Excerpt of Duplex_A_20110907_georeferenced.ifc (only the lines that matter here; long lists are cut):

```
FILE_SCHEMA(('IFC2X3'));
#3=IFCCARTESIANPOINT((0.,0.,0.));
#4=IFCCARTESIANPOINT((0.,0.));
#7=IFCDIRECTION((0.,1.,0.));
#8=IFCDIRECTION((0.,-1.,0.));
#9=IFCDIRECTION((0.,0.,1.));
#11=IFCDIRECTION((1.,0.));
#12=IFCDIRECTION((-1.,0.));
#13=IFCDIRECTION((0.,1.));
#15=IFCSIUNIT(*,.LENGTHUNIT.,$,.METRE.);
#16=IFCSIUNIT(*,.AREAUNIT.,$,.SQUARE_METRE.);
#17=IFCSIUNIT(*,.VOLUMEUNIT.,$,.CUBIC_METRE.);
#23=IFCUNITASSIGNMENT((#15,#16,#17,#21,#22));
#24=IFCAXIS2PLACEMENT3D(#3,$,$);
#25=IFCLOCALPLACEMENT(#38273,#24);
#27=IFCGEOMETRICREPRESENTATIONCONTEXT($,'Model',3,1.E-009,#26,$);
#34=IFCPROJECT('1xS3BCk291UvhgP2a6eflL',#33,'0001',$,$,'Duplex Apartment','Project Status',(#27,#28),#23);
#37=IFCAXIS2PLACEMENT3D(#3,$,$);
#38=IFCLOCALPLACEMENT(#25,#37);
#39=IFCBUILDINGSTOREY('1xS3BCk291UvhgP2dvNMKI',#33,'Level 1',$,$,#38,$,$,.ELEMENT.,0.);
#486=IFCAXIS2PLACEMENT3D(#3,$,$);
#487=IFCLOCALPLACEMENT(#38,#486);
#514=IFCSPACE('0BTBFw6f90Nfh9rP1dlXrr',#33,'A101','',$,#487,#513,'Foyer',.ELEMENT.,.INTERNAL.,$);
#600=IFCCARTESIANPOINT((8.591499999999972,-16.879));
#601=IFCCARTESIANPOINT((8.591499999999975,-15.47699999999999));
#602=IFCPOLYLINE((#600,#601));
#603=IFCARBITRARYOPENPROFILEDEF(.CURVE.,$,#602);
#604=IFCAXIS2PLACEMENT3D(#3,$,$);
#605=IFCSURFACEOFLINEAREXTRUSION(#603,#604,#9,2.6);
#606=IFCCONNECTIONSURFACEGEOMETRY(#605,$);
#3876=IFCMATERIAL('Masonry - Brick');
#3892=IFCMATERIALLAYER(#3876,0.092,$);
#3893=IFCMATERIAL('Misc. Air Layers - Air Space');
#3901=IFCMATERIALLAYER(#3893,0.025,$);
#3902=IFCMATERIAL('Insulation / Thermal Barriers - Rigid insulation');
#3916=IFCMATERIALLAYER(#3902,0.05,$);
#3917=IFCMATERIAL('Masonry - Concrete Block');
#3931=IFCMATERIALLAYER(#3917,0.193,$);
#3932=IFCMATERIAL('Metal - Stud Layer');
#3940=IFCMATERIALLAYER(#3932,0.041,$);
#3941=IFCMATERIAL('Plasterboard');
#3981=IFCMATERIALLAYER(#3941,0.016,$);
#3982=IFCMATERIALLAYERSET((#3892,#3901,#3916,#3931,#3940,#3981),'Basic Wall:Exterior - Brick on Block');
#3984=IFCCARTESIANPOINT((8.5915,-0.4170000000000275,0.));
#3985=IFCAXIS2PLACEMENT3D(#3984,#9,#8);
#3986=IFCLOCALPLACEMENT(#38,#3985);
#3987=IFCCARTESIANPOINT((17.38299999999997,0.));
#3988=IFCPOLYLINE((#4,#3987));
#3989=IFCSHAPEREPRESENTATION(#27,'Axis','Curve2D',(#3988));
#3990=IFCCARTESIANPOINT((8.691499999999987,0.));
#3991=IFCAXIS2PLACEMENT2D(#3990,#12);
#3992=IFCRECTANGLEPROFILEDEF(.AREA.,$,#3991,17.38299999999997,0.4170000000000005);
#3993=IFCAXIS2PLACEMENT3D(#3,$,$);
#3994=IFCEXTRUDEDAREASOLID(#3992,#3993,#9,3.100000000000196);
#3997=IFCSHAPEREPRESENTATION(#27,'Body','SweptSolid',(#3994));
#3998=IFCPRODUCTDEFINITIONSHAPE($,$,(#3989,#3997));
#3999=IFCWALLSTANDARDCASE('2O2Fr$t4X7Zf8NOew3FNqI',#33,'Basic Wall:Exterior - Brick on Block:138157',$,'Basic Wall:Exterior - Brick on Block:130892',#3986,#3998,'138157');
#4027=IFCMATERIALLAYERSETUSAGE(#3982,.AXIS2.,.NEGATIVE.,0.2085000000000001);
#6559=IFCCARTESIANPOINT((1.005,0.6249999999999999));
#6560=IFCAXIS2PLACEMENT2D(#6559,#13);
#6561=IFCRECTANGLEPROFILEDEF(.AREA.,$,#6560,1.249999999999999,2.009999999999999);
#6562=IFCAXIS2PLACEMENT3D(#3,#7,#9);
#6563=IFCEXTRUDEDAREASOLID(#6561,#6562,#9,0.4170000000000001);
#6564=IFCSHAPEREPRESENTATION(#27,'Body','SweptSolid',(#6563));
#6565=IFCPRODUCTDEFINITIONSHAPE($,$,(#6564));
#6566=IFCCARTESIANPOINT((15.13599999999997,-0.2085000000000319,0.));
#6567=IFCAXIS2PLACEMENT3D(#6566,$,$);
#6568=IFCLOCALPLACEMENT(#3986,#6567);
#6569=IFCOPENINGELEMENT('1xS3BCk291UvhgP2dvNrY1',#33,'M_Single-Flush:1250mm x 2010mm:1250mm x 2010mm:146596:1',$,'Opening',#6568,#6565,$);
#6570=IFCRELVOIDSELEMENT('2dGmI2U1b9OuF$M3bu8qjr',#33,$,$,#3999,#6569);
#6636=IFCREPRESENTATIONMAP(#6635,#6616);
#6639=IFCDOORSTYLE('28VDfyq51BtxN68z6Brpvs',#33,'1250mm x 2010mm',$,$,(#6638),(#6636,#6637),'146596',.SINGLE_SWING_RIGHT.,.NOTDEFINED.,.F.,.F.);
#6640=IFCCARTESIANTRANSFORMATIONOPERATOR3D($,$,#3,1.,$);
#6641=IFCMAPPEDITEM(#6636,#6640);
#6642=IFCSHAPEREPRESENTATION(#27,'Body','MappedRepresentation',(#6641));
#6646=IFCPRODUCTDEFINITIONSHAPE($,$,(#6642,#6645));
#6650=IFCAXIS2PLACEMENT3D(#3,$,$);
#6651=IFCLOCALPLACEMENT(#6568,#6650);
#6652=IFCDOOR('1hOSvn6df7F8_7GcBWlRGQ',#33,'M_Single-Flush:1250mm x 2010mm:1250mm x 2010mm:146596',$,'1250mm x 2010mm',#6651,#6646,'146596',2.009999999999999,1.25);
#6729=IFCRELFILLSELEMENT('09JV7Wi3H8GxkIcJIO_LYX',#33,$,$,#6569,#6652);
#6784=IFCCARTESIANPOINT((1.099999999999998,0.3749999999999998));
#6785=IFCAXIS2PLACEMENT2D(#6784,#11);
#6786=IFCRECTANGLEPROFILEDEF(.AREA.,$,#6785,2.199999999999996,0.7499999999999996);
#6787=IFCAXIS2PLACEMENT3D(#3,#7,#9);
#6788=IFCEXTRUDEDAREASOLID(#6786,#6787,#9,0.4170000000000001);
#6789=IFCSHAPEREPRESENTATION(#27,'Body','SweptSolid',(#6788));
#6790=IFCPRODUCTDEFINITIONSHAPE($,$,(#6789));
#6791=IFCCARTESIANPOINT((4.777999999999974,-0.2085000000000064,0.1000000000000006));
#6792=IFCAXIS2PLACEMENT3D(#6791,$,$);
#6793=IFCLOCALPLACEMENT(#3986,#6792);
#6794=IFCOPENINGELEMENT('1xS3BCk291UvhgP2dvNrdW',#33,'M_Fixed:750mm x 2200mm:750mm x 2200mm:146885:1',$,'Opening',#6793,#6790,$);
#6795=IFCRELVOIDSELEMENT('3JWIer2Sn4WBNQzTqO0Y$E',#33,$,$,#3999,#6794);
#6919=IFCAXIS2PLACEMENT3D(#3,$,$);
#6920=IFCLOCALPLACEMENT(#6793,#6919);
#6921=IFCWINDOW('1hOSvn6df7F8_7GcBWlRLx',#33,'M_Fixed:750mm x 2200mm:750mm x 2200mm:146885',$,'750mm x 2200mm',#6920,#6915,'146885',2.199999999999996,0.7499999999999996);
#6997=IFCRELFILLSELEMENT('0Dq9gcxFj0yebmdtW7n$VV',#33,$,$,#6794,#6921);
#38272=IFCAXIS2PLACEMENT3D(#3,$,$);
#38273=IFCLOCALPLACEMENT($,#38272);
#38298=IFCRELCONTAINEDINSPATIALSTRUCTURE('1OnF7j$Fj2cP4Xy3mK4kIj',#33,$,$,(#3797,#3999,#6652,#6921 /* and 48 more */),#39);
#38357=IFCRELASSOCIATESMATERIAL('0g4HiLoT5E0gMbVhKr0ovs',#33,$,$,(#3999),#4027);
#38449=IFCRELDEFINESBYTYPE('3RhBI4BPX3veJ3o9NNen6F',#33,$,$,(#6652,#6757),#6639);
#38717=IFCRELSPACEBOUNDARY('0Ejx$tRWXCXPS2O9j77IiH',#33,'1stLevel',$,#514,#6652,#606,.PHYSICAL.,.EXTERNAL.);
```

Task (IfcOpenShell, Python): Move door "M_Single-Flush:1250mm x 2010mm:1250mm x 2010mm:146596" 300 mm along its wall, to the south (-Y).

```python
import numpy as np
import ifcopenshell
import ifcopenshell.api.geometry
import ifcopenshell.util.placement

model = ifcopenshell.open("Duplex_A_20110907_georeferenced.ifc")

door = model.by_id(6652)
opening = door.FillsVoids[0].RelatingOpeningElement
wall = opening.VoidsElements[0].RelatingBuildingElement

wall_matrix = ifcopenshell.util.placement.get_local_placement(wall.ObjectPlacement)
shift = wall_matrix[:3, 0] * 0.3
before = ifcopenshell.util.placement.get_local_placement(door.ObjectPlacement)[:3, 3].copy()

# The door is placed relative to its opening, so it follows when the opening moves.
matrix = ifcopenshell.util.placement.get_local_placement(opening.ObjectPlacement)
matrix[:3, 3] += shift
ifcopenshell.api.geometry.edit_object_placement(
    model, product=opening, matrix=matrix, is_si=False, should_transform_children=True
)

# Space boundary surfaces are stored in each space's coordinates; move them too.
for rel in door.ProvidesBoundaries:
    if not rel.ConnectionGeometry:
        continue
    surface = rel.ConnectionGeometry.SurfaceOnRelatingElement
    space_matrix = ifcopenshell.util.placement.get_local_placement(rel.RelatingSpace.ObjectPlacement)
    point = np.array(surface.Position.Location.Coordinates) + space_matrix[:3, :3].T @ shift
    surface.Position = model.createIfcAxis2Placement3D(
        model.createIfcCartesianPoint(point.tolist()), surface.Position.Axis, surface.Position.RefDirection
    )

after = ifcopenshell.util.placement.get_local_placement(door.ObjectPlacement)[:3, 3]
print("door moved by", (after - before).round(3) + 0.0)

model.write("Duplex_A_20110907_georeferenced_rev.ifc")
```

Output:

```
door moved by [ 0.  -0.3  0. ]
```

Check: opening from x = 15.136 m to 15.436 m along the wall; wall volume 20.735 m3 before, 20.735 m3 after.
